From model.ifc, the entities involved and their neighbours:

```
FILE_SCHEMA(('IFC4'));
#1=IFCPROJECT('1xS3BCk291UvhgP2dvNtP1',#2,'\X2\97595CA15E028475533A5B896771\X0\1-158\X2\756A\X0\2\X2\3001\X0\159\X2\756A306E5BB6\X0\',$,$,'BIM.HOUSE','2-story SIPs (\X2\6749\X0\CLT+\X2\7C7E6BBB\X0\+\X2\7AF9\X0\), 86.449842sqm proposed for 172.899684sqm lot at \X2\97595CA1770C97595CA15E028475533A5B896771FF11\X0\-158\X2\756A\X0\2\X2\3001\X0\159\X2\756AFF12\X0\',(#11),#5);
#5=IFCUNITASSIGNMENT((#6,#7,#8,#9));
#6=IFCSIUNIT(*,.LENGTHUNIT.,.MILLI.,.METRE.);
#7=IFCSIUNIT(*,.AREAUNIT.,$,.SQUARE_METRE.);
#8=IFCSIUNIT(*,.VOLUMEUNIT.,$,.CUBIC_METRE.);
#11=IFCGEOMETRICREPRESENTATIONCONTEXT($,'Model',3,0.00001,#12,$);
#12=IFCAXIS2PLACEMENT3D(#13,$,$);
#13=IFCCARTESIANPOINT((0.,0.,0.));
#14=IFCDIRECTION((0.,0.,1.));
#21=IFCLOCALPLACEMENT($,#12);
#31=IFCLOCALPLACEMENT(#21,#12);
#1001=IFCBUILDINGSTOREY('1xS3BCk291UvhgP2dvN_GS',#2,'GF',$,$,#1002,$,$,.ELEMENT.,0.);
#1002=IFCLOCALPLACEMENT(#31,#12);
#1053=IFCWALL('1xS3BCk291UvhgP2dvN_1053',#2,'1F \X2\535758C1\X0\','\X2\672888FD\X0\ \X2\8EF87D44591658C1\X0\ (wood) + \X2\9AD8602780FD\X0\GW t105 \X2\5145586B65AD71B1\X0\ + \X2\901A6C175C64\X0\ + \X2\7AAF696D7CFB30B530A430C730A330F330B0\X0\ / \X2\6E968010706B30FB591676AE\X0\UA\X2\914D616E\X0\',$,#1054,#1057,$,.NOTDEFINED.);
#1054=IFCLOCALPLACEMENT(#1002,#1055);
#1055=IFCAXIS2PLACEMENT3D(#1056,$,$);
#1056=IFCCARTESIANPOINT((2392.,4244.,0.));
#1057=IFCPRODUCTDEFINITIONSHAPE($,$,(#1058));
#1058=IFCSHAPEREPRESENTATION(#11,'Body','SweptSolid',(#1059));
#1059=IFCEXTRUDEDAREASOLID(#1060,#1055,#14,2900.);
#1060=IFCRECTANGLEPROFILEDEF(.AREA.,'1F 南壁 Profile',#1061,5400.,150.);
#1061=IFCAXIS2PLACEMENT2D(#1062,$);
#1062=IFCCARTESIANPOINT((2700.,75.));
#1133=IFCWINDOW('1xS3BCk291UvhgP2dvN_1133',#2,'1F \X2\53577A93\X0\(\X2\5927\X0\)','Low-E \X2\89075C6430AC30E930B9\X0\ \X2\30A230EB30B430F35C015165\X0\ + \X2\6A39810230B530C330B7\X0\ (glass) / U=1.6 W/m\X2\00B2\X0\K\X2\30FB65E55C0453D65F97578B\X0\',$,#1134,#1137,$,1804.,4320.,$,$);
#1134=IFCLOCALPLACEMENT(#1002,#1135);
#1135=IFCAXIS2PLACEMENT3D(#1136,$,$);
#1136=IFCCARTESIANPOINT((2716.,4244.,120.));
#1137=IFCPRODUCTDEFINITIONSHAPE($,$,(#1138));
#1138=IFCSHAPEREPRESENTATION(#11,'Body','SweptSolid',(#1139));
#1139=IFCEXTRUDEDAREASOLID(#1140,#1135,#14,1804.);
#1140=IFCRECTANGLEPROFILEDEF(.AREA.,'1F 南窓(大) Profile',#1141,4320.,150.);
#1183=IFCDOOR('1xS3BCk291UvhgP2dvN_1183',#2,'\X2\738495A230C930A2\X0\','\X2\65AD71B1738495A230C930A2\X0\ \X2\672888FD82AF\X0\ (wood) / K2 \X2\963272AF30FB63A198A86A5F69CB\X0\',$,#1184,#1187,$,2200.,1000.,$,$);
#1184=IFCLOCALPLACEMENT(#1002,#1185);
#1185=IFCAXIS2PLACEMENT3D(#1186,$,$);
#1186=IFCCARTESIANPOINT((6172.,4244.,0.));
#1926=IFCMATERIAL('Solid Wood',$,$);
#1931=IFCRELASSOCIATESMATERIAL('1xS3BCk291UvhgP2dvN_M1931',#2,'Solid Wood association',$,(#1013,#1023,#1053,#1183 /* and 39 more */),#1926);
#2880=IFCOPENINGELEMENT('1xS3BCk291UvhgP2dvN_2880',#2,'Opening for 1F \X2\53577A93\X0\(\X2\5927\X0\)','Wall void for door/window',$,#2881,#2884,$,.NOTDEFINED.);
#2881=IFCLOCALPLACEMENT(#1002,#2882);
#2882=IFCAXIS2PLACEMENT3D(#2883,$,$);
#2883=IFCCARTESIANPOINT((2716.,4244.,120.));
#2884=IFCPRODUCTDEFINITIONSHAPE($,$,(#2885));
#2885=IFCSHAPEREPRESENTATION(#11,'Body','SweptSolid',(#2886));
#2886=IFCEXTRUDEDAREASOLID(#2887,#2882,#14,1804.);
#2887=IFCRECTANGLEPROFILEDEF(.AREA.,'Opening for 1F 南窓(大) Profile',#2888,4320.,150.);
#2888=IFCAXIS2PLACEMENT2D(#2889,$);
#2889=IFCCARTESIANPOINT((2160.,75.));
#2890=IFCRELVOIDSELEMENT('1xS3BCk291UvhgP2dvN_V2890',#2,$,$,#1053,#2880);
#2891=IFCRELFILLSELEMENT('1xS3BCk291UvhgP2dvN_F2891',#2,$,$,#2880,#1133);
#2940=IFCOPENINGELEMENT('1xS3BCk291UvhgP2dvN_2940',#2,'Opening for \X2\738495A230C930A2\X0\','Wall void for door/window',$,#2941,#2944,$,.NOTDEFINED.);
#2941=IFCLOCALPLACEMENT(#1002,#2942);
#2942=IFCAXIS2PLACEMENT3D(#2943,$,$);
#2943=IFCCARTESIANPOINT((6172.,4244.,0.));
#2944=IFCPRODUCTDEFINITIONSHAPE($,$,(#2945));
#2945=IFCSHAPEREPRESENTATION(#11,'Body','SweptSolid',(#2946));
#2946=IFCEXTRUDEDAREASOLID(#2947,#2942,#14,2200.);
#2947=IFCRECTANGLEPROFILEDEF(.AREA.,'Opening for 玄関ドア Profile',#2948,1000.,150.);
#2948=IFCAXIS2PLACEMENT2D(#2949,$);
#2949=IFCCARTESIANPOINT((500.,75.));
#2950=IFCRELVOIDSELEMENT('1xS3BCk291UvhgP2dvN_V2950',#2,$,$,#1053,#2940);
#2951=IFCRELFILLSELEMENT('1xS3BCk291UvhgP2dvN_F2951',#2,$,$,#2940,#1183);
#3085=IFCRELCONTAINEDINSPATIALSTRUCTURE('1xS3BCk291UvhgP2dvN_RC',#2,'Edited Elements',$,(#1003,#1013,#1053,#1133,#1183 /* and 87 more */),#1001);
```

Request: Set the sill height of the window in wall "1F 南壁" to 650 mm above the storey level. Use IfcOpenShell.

```python
import numpy as np
import ifcopenshell
import ifcopenshell.api.geometry
import ifcopenshell.geom
import ifcopenshell.util.element
import ifcopenshell.util.placement
import ifcopenshell.util.shape
import ifcopenshell.util.unit

model = ifcopenshell.open("model.ifc")
unit_scale = ifcopenshell.util.unit.calculate_unit_scale(model)

window = model.by_guid("1xS3BCk291UvhgP2dvN_1133")
opening = window.FillsVoids[0].RelatingOpeningElement
storey = ifcopenshell.util.element.get_container(window, ifc_class="IfcBuildingStorey")
level = ifcopenshell.util.placement.get_local_placement(storey.ObjectPlacement)[2, 3]

# The opening's origin need not be at the sill, so measure its lowest point.
shape = ifcopenshell.geom.create_shape(ifcopenshell.geom.settings(), opening)
bottom = ifcopenshell.util.shape.get_shape_bottom_elevation(shape, shape.geometry) / unit_scale
dz = level + 0.65 / unit_scale - bottom

shift = np.array([0.0, 0.0, dz])
# The window is not placed relative to its opening, so move both.
for product in (opening, window):
    matrix = ifcopenshell.util.placement.get_local_placement(product.ObjectPlacement)
    matrix[:3, 3] += shift
    ifcopenshell.api.geometry.edit_object_placement(model, product=product, matrix=matrix, is_si=False)

print(f"moved by {dz * unit_scale:+.3f} m")

model.write("model-out.ifc")
```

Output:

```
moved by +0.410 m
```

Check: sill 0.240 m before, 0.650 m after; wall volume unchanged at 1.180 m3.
